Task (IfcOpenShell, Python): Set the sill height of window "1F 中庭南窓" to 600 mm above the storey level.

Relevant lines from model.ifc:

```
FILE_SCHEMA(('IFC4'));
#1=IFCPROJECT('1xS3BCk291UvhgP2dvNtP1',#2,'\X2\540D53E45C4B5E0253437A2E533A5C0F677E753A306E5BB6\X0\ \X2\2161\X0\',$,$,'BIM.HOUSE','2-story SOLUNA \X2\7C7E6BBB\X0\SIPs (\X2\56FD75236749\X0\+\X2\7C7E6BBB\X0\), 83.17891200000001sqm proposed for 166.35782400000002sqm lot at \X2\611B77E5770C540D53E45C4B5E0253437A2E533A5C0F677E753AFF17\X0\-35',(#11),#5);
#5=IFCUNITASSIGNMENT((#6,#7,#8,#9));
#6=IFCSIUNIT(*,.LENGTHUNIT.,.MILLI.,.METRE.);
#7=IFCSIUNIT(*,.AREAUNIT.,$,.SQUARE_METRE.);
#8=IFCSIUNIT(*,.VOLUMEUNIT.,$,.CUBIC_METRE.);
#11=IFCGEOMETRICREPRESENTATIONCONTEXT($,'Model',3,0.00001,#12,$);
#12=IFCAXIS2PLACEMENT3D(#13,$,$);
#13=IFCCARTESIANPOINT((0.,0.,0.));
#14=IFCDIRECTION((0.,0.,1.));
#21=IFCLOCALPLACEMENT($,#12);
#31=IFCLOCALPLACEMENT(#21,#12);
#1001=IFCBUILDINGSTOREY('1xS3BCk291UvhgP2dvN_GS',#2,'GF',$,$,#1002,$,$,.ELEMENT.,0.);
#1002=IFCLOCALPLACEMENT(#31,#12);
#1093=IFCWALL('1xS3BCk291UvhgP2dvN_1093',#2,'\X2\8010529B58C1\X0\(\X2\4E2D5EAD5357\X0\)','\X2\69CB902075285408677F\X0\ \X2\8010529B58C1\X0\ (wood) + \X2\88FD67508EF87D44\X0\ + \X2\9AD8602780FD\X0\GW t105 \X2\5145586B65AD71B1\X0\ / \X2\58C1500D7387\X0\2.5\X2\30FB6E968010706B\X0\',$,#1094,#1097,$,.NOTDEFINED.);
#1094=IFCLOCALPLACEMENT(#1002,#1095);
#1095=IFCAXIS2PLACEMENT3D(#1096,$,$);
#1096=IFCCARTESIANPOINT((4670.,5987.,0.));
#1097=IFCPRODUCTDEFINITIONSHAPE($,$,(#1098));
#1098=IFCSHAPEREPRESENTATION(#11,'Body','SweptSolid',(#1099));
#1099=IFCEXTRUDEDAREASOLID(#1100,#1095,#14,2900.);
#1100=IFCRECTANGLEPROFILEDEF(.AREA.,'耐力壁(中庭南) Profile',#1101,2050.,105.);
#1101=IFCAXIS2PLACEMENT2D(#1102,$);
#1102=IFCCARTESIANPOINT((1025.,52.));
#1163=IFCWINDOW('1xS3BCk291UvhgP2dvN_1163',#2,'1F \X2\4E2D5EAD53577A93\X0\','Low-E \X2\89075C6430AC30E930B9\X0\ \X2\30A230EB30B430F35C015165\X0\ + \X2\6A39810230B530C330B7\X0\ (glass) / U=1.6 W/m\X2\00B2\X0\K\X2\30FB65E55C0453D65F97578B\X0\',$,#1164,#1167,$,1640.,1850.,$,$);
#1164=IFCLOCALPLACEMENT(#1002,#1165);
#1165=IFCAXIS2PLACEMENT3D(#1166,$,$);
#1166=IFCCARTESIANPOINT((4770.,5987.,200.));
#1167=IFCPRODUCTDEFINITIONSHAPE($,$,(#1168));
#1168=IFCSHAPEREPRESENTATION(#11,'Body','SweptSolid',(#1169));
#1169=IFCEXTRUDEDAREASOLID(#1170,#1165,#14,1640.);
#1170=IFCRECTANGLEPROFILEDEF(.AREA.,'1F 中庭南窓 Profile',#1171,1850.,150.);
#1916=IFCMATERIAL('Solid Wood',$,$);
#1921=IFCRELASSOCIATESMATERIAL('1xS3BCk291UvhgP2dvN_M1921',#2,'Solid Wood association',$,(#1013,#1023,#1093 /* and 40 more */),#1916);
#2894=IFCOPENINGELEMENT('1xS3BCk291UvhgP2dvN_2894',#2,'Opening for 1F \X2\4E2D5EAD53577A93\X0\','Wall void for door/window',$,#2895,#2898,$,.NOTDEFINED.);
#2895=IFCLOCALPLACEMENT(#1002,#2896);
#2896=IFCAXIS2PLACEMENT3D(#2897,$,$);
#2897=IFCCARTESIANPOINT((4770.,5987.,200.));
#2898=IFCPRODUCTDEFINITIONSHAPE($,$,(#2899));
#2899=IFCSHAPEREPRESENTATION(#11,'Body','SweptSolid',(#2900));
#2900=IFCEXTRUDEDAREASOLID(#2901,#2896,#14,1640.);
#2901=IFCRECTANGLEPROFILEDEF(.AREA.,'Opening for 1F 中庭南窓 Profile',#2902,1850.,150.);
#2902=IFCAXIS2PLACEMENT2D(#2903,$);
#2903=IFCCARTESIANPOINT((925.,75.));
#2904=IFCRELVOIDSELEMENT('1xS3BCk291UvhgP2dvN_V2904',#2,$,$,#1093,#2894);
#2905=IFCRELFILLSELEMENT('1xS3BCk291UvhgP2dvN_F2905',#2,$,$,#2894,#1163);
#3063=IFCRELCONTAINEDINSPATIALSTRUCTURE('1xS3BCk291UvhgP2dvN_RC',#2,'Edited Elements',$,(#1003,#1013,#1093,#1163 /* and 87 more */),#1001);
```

```python
import numpy as np
import ifcopenshell
import ifcopenshell.api.geometry
import ifcopenshell.geom
import ifcopenshell.util.element
import ifcopenshell.util.placement
import ifcopenshell.util.shape
import ifcopenshell.util.unit

model = ifcopenshell.open("model.ifc")
unit_scale = ifcopenshell.util.unit.calculate_unit_scale(model)

window = model.by_guid("1xS3BCk291UvhgP2dvN_1163")
opening = window.FillsVoids[0].RelatingOpeningElement
storey = ifcopenshell.util.element.get_container(window, ifc_class="IfcBuildingStorey")
level = ifcopenshell.util.placement.get_local_placement(storey.ObjectPlacement)[2, 3]

# The opening's origin need not be at the sill, so measure its lowest point.
shape = ifcopenshell.geom.create_shape(ifcopenshell.geom.settings(), opening)
bottom = ifcopenshell.util.shape.get_shape_bottom_elevation(shape, shape.geometry) / unit_scale
dz = level + 600.0 - bottom

shift = np.array([0.0, 0.0, dz])
# The window is not placed relative to its opening, so move both.
for product in (opening, window):
    matrix = ifcopenshell.util.placement.get_local_placement(product.ObjectPlacement)
    matrix[:3, 3] += shift
    ifcopenshell.api.geometry.edit_object_placement(model, product=product, matrix=matrix, is_si=False)

print(f"moved by {dz * unit_scale:+.3f} m")

model.write("model_edited.ifc")
```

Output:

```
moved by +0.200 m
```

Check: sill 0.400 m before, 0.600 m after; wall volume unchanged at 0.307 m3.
